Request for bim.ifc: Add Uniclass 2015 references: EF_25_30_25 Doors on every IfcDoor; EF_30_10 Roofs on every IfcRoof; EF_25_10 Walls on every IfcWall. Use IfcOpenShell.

First a look at what the model holds.

```python
import ifcopenshell

model = ifcopenshell.open("bim.ifc")
print(model.schema)
print("classifications:", [c.Name for c in model.by_type("IfcClassification")])
for ifc_class in ("IfcDoor", "IfcRoof", "IfcStair", "IfcWall", "IfcWindow"):
    print(ifc_class, len(model.by_type(ifc_class)))
```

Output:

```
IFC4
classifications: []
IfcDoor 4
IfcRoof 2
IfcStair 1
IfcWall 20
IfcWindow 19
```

```python
import ifcopenshell
import ifcopenshell.api.classification

model = ifcopenshell.open("bim.ifc")

system = ifcopenshell.api.classification.add_classification(model, classification="Uniclass 2015")

codes = {
    "IfcDoor": ("EF_25_30_25", "Doors"),
    "IfcRoof": ("EF_30_10", "Roofs"),
    "IfcWall": ("EF_25_10", "Walls"),
}
for ifc_class, (code, name) in codes.items():
    products = model.by_type(ifc_class)
    ifcopenshell.api.classification.add_reference(
        model, products=products, classification=system, identification=code, name=name
    )
    print(code, len(products))

model.write("bim_rev.ifc")
```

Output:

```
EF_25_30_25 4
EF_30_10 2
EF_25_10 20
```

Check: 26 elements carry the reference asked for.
